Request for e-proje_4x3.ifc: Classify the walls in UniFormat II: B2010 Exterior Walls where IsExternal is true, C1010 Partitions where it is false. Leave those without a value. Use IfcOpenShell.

First a look at what the model holds.

```python
import ifcopenshell
import ifcopenshell.util.element

model = ifcopenshell.open("e-proje_4x3.ifc")
print(model.schema)
print("classifications:", [c.Name for c in model.by_type("IfcClassification")])
values = [ifcopenshell.util.element.get_pset(e, "Pset_WallCommon", "IsExternal") for e in model.by_type("IfcWall")]
for value in (True, False, None):
    print("IsExternal", value, values.count(value))
```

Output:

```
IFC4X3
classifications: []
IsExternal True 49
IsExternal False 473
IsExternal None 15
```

```python
import ifcopenshell
import ifcopenshell.api.classification
import ifcopenshell.util.element

model = ifcopenshell.open("e-proje_4x3.ifc")

system = ifcopenshell.api.classification.add_classification(model, classification="UniFormat II")

walls = model.by_type("IfcWall")
external = {e: ifcopenshell.util.element.get_pset(e, "Pset_WallCommon", "IsExternal") for e in walls}
for flag, code, name in ((True, "B2010", "Exterior Walls"), (False, "C1010", "Partitions")):
    products = [e for e in walls if external[e] is flag]
    ifcopenshell.api.classification.add_reference(
        model, products=products, classification=system, identification=code, name=name
    )
    print(code, len(products))

model.write("e-proje_4x3-out.ifc")
```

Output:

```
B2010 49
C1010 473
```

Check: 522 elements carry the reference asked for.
